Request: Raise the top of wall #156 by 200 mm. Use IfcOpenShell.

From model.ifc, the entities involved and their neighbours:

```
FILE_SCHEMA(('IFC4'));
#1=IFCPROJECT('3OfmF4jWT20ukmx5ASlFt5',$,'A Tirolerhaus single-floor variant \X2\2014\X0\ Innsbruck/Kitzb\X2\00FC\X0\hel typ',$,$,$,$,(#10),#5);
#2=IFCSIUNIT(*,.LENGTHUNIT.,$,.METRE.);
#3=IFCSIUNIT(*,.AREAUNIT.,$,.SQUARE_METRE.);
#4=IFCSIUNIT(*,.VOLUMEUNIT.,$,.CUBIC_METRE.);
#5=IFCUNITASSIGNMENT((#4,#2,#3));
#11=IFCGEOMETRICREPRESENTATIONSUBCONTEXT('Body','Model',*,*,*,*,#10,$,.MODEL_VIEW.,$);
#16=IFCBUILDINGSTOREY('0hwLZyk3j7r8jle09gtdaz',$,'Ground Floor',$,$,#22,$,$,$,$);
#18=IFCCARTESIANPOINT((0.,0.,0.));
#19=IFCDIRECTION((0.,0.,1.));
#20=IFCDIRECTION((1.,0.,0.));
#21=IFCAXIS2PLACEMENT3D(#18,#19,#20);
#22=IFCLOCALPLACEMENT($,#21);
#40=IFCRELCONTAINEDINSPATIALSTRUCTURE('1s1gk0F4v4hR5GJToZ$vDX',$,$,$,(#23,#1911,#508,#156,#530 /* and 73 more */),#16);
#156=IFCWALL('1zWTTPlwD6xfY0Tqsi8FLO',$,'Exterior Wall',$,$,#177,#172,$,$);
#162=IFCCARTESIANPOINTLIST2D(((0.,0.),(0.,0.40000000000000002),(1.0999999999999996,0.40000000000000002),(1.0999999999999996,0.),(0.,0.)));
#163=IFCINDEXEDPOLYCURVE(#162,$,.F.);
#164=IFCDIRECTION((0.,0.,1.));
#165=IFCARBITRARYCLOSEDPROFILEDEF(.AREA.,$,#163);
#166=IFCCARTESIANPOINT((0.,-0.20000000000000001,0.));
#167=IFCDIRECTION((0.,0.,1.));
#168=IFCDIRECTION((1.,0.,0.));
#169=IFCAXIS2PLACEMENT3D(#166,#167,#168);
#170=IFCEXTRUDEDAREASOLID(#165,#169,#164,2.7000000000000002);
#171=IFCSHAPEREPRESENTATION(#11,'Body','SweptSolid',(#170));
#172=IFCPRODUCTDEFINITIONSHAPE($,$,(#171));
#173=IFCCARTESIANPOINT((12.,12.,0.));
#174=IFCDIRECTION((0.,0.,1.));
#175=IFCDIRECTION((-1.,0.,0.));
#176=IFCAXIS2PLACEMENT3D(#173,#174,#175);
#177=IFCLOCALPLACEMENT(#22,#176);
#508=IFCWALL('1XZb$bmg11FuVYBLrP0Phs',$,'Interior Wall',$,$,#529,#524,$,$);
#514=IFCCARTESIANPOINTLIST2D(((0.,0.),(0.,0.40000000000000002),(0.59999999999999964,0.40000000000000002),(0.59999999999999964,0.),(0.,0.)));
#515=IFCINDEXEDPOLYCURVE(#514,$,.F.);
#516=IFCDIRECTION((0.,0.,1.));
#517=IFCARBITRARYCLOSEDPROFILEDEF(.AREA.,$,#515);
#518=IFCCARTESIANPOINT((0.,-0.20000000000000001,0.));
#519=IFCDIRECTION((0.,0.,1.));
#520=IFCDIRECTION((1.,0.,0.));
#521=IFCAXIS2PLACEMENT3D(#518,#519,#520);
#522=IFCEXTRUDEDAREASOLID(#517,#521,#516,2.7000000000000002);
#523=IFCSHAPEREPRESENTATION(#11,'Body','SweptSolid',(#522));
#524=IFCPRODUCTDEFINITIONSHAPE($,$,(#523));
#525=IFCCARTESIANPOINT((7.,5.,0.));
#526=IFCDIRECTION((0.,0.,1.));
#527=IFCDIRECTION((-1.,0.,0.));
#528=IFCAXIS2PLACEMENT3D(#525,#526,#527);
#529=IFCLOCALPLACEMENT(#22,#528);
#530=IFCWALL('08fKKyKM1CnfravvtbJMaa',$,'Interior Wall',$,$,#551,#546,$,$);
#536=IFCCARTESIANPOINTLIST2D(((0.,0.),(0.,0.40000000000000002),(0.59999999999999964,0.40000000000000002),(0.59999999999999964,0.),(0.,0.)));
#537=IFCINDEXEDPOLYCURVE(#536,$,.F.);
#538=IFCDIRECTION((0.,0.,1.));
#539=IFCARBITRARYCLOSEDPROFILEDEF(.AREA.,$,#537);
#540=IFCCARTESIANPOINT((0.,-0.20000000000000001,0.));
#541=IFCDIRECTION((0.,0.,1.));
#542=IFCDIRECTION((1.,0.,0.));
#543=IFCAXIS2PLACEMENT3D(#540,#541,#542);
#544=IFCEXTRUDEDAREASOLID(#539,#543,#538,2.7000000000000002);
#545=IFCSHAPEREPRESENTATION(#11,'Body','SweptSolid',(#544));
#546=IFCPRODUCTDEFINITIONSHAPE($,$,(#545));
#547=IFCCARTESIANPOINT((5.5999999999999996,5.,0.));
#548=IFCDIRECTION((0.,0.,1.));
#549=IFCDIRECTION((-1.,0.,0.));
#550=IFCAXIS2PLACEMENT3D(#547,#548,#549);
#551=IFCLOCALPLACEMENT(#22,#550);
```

```python
import ifcopenshell
import ifcopenshell.geom
import ifcopenshell.util.representation
import ifcopenshell.util.shape

model = ifcopenshell.open("model.ifc")
settings = ifcopenshell.geom.settings()


def volume(element):
    """Net volume in cubic metres, openings subtracted."""
    shape = ifcopenshell.geom.create_shape(settings, element)
    return ifcopenshell.util.shape.get_volume(shape.geometry)


wall = model.by_id(156)
before = volume(wall)

body = ifcopenshell.util.representation.get_representation(wall, "Model", "Body")
solid = body.Items[0]
old_height = solid.Depth
solid.Depth += 0.2
after = volume(wall)

print(f"height {old_height:g} -> {solid.Depth:g}, volume {before:.3f} -> {after:.3f} m3")

model.write("model_updated.ifc")
```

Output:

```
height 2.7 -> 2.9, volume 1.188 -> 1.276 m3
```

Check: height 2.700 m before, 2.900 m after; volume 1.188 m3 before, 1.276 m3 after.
